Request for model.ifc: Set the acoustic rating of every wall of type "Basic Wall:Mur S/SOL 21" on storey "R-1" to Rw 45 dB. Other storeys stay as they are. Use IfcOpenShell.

First a look at what the model holds.

```python
import ifcopenshell
import ifcopenshell.util.element

model = ifcopenshell.open("model.ifc")
print(model.schema)
storey = next(s for s in model.by_type("IfcBuildingStorey") if s.Name == "R-1")
walls = [e for e in ifcopenshell.util.element.get_decomposition(storey) if e.is_a("IfcWall")]
seen = {}
for e in walls:
    element_type = ifcopenshell.util.element.get_type(e)
    key = (element_type.Name if element_type != e and element_type else None, ifcopenshell.util.element.get_pset(e, "Pset_WallCommon", "AcousticRating"))
    seen[key] = seen.get(key, 0) + 1
for (name, value), count in sorted(seen.items(), key=str):
    print(count, "x", name, "|", value)
```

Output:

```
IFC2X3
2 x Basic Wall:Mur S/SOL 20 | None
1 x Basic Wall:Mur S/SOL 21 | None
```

```python
import ifcopenshell
import ifcopenshell.api.pset
import ifcopenshell.util.element

model = ifcopenshell.open("model.ifc")

storey = next(s for s in model.by_type("IfcBuildingStorey") if s.Name == "R-1")
walls = [e for e in ifcopenshell.util.element.get_decomposition(storey) if e.is_a("IfcWall")]

count = 0
for e in walls:
    element_type = ifcopenshell.util.element.get_type(e)
    if element_type in (None, e) or element_type.Name != "Basic Wall:Mur S/SOL 21":
        continue
    # add_pset returns the element's existing set when there is one.
    pset = ifcopenshell.api.pset.add_pset(model, product=e, name="Pset_WallCommon")
    ifcopenshell.api.pset.edit_pset(model, pset=pset, properties={"AcousticRating": "Rw 45 dB"})
    count += 1

print(count, "walls updated")

model.write("model-out.ifc")
```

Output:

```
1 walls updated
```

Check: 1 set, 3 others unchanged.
